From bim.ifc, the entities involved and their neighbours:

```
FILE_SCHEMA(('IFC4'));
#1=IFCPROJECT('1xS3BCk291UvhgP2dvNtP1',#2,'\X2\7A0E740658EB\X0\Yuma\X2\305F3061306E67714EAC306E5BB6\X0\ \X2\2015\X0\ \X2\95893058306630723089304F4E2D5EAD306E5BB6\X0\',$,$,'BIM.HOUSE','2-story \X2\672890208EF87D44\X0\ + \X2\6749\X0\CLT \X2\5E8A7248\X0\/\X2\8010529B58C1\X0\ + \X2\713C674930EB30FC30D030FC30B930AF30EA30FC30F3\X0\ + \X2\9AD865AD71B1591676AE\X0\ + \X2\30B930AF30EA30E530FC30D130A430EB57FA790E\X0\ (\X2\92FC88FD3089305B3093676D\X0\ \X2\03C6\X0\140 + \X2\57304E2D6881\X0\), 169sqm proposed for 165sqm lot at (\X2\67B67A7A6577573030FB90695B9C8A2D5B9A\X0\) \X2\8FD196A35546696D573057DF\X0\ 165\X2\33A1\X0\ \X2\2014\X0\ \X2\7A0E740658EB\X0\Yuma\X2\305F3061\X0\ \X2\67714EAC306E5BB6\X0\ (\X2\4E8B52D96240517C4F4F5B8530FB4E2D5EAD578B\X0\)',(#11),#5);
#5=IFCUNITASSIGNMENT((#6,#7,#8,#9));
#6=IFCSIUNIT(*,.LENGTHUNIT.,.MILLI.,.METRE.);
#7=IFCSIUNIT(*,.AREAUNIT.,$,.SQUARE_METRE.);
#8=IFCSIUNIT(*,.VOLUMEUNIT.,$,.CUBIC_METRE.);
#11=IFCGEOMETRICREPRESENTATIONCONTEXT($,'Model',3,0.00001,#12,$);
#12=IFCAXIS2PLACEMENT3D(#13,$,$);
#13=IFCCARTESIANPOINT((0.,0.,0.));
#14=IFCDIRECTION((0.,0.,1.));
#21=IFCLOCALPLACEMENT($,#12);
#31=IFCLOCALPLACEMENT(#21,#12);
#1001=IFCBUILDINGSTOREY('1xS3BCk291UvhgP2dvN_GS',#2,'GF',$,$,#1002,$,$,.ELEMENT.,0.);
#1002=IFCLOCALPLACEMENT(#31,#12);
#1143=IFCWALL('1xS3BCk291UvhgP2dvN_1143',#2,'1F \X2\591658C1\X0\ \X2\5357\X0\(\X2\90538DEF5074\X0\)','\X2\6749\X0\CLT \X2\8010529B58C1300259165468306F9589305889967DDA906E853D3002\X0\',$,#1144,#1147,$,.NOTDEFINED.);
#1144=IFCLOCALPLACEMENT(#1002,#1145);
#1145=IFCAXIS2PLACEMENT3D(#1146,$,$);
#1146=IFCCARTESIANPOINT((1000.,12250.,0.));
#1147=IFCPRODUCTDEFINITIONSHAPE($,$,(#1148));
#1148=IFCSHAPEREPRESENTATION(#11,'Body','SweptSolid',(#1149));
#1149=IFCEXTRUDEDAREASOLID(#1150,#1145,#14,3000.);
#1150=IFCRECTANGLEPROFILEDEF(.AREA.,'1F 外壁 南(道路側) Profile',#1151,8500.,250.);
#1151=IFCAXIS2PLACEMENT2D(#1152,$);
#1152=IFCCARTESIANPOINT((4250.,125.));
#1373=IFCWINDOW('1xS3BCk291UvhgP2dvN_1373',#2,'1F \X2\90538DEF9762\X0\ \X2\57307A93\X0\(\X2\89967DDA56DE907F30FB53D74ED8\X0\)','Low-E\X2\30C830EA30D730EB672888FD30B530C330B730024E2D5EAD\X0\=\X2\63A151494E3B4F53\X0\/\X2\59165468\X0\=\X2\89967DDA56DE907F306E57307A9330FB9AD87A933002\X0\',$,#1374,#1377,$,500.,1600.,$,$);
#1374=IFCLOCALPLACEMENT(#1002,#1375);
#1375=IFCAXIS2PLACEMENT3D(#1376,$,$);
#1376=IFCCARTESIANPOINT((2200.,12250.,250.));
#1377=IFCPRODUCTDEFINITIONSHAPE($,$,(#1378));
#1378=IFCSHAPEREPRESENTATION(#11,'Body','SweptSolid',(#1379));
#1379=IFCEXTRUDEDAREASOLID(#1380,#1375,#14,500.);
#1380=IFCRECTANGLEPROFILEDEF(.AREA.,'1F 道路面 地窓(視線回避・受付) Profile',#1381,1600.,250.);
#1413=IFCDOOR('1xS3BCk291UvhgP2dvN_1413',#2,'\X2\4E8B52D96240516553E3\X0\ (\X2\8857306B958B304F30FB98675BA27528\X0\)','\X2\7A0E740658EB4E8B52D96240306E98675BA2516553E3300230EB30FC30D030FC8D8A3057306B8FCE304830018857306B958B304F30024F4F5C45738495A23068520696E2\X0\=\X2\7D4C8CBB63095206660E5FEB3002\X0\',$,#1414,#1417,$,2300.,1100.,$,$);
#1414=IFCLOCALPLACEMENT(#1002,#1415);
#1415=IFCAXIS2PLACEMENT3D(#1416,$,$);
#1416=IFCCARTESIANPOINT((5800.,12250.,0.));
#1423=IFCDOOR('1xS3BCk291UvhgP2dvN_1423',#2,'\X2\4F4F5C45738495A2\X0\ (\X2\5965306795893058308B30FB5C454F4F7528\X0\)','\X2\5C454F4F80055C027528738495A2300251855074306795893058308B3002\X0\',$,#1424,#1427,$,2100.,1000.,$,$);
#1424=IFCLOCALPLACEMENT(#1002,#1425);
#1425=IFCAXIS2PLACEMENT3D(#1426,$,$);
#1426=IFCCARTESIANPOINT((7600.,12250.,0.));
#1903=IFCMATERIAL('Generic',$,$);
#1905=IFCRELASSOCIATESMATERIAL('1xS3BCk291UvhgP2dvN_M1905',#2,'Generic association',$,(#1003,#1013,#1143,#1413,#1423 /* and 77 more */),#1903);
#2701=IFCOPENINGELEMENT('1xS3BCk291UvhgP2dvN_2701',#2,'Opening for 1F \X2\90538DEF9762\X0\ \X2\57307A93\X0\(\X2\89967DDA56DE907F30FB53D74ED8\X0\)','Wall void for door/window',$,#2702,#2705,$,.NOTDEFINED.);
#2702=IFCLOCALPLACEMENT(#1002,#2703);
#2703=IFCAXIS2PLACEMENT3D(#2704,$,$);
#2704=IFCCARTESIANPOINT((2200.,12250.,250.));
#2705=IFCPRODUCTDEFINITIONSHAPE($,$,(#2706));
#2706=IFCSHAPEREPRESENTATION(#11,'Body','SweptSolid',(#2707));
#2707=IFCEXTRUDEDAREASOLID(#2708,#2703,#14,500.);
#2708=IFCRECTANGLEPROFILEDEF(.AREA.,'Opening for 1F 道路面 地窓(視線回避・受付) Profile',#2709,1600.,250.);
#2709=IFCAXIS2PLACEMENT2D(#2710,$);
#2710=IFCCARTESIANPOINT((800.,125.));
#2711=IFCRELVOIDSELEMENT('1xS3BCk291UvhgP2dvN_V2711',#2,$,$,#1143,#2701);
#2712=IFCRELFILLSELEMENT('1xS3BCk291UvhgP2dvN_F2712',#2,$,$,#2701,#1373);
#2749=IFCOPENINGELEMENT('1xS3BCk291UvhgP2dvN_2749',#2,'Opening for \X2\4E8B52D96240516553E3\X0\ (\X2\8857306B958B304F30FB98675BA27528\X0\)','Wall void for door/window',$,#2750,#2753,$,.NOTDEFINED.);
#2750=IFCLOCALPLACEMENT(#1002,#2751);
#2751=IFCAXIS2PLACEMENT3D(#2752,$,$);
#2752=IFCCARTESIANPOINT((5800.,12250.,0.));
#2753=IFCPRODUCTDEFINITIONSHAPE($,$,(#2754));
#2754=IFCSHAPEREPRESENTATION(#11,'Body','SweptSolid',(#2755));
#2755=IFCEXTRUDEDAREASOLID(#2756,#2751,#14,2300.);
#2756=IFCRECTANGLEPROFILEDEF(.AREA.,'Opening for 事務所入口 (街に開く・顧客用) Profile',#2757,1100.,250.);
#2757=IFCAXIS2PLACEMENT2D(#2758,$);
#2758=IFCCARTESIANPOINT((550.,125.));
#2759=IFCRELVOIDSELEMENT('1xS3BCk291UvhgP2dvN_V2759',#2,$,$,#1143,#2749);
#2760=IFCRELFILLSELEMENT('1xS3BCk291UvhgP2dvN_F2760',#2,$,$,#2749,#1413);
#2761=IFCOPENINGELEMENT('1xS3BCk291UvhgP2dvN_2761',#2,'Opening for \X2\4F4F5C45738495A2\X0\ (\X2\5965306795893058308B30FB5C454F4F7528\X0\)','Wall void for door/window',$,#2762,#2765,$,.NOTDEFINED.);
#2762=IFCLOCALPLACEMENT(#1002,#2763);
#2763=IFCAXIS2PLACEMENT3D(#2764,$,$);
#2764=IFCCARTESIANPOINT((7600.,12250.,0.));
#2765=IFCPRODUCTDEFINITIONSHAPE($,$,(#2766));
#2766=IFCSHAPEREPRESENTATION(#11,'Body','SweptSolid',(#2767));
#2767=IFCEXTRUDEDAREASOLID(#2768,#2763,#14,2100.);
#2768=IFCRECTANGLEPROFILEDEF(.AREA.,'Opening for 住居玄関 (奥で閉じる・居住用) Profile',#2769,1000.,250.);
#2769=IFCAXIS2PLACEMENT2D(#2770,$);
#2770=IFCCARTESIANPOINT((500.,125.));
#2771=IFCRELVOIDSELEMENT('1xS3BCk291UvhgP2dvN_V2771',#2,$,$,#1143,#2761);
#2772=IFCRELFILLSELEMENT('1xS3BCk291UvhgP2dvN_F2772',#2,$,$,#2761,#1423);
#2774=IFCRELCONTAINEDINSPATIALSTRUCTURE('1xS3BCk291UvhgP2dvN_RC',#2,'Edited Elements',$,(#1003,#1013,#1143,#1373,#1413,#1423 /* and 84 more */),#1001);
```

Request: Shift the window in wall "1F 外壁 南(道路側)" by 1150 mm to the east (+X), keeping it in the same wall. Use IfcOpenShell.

```python
import ifcopenshell
import ifcopenshell.api.geometry
import ifcopenshell.util.placement
import ifcopenshell.util.unit

model = ifcopenshell.open("bim.ifc")
unit_scale = ifcopenshell.util.unit.calculate_unit_scale(model)

window = model.by_guid("1xS3BCk291UvhgP2dvN_1373")
opening = window.FillsVoids[0].RelatingOpeningElement
wall = opening.VoidsElements[0].RelatingBuildingElement

wall_matrix = ifcopenshell.util.placement.get_local_placement(wall.ObjectPlacement)
shift = wall_matrix[:3, 0] * 1.15 / unit_scale
before = ifcopenshell.util.placement.get_local_placement(window.ObjectPlacement)[:3, 3].copy()

# The window is not placed relative to its opening, so move both.
for product in (opening, window):
    matrix = ifcopenshell.util.placement.get_local_placement(product.ObjectPlacement)
    matrix[:3, 3] += shift
    ifcopenshell.api.geometry.edit_object_placement(model, product=product, matrix=matrix, is_si=False)

after = ifcopenshell.util.placement.get_local_placement(window.ObjectPlacement)[:3, 3]
print("window moved by", (after - before).round(3) + 0.0)

model.write("bim_v2.ifc")
```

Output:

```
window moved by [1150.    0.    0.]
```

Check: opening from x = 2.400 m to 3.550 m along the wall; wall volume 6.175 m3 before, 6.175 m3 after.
